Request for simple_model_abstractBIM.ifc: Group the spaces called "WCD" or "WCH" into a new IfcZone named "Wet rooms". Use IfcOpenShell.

First a look at what the model holds.

```python
import ifcopenshell

model = ifcopenshell.open("simple_model_abstractBIM.ifc")
print(model.schema)
seen = {}
for space in model.by_type("IfcSpace"):
    seen[space.LongName] = seen.get(space.LongName, 0) + 1
for name, count in sorted(seen.items(), key=str):
    print(count, "x", name)
print("zones:", [z.Name for z in model.by_type("IfcZone")][:20])
```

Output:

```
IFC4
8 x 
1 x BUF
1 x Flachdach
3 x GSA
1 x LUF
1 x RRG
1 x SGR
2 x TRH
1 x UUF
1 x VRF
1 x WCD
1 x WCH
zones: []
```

```python
import ifcopenshell
import ifcopenshell.api.group
import ifcopenshell.api.root

model = ifcopenshell.open("simple_model_abstractBIM.ifc")

names = {"WCD", "WCH"}
spaces = [s for s in model.by_type("IfcSpace") if s.LongName in names]

zone = ifcopenshell.api.root.create_entity(model, ifc_class="IfcZone", name="Wet rooms")
ifcopenshell.api.group.assign_group(model, products=spaces, group=zone)
print(len(spaces), "spaces in", zone.Name)

model.write("simple_model_abstractBIM_updated.ifc")
```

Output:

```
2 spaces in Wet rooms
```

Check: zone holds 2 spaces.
